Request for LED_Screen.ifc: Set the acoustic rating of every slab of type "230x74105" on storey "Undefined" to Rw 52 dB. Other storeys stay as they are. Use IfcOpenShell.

First a look at what the model holds.

```python
import ifcopenshell
import ifcopenshell.util.element

model = ifcopenshell.open("LED_Screen.ifc")
print(model.schema)
storey = next(s for s in model.by_type("IfcBuildingStorey") if s.Name == "Undefined")
slabs = [e for e in ifcopenshell.util.element.get_decomposition(storey) if e.is_a("IfcSlab")]
seen = {}
for e in slabs:
    element_type = ifcopenshell.util.element.get_type(e)
    key = (element_type.Name if element_type != e and element_type else None, ifcopenshell.util.element.get_pset(e, "Pset_SlabCommon", "AcousticRating"))
    seen[key] = seen.get(key, 0) + 1
for (name, value), count in sorted(seen.items(), key=str):
    print(count, "x", name, "|", value)
```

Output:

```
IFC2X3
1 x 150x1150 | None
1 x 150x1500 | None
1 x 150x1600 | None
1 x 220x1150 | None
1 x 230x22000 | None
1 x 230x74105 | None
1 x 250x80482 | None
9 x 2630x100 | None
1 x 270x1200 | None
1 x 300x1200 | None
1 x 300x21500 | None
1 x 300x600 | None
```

```python
import ifcopenshell
import ifcopenshell.api.pset
import ifcopenshell.util.element

model = ifcopenshell.open("LED_Screen.ifc")

storey = next(s for s in model.by_type("IfcBuildingStorey") if s.Name == "Undefined")
slabs = [e for e in ifcopenshell.util.element.get_decomposition(storey) if e.is_a("IfcSlab")]

count = 0
for e in slabs:
    element_type = ifcopenshell.util.element.get_type(e)
    if element_type in (None, e) or element_type.Name != "230x74105":
        continue
    found = ifcopenshell.util.element.get_pset(e, "Pset_SlabCommon", should_inherit=False)
    if found:
        pset = model.by_id(found["id"])
        if len(ifcopenshell.util.element.get_elements_by_pset(pset)) > 1:
            pset = ifcopenshell.api.pset.unshare_pset(model, products=[e], pset=pset)[0]
    else:
        pset = ifcopenshell.api.pset.add_pset(model, product=e, name="Pset_SlabCommon")
    ifcopenshell.api.pset.edit_pset(model, pset=pset, properties={"AcousticRating": "Rw 52 dB"})
    count += 1

print(count, "slabs updated")

model.write("LED_Screen-out.ifc")
```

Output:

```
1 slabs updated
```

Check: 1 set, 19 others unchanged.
